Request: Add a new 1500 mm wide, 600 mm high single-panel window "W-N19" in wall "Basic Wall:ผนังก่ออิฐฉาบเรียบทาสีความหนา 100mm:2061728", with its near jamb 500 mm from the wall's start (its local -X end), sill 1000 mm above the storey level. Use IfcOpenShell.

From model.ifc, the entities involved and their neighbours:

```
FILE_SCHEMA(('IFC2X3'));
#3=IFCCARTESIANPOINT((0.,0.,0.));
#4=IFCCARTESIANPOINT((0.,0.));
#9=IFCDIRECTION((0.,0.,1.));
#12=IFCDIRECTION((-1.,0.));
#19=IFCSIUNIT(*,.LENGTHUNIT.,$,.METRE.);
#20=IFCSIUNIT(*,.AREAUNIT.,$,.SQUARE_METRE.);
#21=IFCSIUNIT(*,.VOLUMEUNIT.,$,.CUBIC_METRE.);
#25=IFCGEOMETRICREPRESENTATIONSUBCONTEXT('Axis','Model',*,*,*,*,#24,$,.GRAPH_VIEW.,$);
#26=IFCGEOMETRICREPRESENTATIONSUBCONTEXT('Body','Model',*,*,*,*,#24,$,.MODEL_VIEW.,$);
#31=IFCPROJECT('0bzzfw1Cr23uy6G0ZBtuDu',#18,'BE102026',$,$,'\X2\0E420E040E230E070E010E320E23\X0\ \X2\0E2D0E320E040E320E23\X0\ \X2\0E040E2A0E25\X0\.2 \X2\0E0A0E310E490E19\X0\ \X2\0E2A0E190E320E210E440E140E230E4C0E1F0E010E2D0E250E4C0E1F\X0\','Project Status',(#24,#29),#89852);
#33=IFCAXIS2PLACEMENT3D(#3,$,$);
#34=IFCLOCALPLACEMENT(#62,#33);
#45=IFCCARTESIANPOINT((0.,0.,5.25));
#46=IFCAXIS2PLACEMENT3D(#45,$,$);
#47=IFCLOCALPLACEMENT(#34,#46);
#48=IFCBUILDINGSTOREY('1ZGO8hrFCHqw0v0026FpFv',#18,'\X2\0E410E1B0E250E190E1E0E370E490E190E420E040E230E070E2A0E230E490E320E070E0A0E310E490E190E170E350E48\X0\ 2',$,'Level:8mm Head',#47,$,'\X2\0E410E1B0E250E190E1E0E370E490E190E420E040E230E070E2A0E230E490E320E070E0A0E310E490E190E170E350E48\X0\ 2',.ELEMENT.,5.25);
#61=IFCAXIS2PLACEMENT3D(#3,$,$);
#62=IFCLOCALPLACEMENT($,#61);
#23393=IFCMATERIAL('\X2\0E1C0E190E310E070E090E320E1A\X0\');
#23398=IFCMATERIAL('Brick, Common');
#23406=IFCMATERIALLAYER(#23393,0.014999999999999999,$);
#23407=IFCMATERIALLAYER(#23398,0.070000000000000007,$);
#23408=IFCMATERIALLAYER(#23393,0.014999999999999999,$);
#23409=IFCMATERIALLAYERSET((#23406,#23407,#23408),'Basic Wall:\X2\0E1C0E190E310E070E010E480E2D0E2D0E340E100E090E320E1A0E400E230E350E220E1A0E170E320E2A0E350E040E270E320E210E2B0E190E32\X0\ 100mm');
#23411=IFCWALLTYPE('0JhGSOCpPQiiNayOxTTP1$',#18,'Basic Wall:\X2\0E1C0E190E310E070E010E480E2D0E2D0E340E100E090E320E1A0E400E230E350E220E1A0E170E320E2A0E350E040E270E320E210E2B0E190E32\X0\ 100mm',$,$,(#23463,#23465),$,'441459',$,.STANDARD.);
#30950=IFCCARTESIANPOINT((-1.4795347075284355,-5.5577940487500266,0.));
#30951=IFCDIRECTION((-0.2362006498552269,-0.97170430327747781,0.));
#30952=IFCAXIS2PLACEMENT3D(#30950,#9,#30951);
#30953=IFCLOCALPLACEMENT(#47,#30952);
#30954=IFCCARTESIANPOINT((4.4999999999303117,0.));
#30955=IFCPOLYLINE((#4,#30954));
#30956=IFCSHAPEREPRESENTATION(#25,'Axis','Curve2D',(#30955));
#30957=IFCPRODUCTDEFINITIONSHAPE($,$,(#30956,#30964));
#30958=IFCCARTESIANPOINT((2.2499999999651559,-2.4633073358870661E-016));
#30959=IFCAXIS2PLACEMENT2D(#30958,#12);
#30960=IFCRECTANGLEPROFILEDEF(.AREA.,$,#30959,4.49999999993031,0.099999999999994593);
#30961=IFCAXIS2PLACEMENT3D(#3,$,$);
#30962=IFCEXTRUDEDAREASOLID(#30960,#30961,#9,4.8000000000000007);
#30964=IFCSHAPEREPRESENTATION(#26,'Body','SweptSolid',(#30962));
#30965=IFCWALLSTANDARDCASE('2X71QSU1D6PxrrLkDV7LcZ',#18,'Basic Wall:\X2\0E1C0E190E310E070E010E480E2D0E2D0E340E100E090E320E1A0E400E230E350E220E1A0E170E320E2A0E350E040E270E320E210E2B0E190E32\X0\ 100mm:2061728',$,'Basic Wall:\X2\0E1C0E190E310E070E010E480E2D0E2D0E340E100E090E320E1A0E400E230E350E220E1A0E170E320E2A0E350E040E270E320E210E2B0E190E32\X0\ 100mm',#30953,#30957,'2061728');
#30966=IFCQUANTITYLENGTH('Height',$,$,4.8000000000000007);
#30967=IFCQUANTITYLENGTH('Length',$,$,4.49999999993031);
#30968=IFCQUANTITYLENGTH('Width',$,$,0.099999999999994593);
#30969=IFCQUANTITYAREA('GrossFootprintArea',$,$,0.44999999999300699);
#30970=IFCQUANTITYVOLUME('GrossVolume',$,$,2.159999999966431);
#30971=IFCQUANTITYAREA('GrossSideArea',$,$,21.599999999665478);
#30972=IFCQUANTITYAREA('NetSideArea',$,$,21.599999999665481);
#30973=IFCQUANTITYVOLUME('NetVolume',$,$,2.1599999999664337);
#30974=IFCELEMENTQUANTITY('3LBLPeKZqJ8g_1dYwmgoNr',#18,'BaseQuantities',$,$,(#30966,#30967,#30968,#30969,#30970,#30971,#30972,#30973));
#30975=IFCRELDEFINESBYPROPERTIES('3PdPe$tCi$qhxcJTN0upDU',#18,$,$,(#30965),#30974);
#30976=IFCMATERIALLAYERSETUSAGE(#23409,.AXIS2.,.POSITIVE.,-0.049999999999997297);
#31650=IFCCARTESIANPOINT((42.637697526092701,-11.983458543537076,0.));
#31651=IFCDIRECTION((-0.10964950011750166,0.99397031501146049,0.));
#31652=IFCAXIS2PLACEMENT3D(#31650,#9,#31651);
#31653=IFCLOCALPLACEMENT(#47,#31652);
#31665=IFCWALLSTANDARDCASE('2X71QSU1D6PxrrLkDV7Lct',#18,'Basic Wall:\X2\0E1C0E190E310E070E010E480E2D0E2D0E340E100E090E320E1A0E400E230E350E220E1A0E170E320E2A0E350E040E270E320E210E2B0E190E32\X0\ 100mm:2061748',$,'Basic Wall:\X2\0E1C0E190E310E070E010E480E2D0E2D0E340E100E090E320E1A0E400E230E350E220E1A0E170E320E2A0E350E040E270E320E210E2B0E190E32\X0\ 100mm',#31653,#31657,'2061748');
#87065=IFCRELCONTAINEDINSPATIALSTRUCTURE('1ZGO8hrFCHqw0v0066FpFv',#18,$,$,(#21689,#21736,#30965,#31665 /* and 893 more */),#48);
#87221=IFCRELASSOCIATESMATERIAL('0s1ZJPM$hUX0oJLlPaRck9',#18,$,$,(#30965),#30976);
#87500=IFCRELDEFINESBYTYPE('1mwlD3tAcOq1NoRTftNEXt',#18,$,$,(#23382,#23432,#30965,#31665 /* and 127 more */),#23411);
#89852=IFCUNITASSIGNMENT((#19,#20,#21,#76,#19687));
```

```python
import numpy as np
import ifcopenshell
import ifcopenshell.api.feature
import ifcopenshell.api.geometry
import ifcopenshell.api.pset
import ifcopenshell.api.root
import ifcopenshell.api.spatial
import ifcopenshell.api.type
import ifcopenshell.geom
import ifcopenshell.util.element
import ifcopenshell.util.placement
import ifcopenshell.util.representation
import ifcopenshell.util.shape
import ifcopenshell.util.unit

model = ifcopenshell.open("model.ifc")
unit_scale = ifcopenshell.util.unit.calculate_unit_scale(model)
area_scale = ifcopenshell.util.unit.calculate_unit_scale(model, "AREAUNIT")
volume_scale = ifcopenshell.util.unit.calculate_unit_scale(model, "VOLUMEUNIT")
settings = ifcopenshell.geom.settings()


def volume(element):
    """Net volume in cubic metres, openings subtracted."""
    shape = ifcopenshell.geom.create_shape(settings, element)
    return ifcopenshell.util.shape.get_volume(shape.geometry)


wall = model.by_guid("2X71QSU1D6PxrrLkDV7LcZ")
storey = ifcopenshell.util.element.get_container(wall, ifc_class="IfcBuildingStorey")
context = ifcopenshell.util.representation.get_context(model, "Model", "Body", "MODEL_VIEW")
before = volume(wall)

width, height, from_end, sill = 1.5, 0.6, 0.5, 1  # metres

# The wall runs along its own X axis, and the end named is its -X end.
wall_shape = ifcopenshell.geom.create_shape(settings, wall)
x, y, z = ifcopenshell.util.shape.get_vertices(wall_shape.geometry).T
start = x.min() + from_end
face, thickness = float(y.min()), float(y.max() - y.min())
wall_matrix = ifcopenshell.util.placement.get_local_placement(wall.ObjectPlacement)
level = ifcopenshell.util.placement.get_local_placement(storey.ObjectPlacement)[2, 3]


def in_wall(x, y):
    """Placement at x, y metres in the wall's axes, at sill height."""
    matrix = wall_matrix.copy()
    matrix[:, 3] = wall_matrix @ np.array([x / unit_scale, y / unit_scale, 0.0, 1.0])
    matrix[2, 3] = level + sill / unit_scale
    return matrix


# Opening: a box that overshoots both wall faces by 50 mm.
opening = ifcopenshell.api.root.create_entity(model, ifc_class="IfcOpeningElement")
box = ifcopenshell.api.geometry.add_wall_representation(
    model, context=context, length=width, height=height, thickness=thickness + 0.1
)
ifcopenshell.api.geometry.assign_representation(model, product=opening, representation=box)
ifcopenshell.api.geometry.edit_object_placement(model, product=opening, matrix=in_wall(start, face - 0.05), is_si=False)
ifcopenshell.api.feature.add_feature(model, feature=opening, element=wall)

window = ifcopenshell.api.root.create_entity(model, ifc_class="IfcWindow", name="W-N19")
window.OverallWidth, window.OverallHeight = width / unit_scale, height / unit_scale
body = ifcopenshell.api.geometry.add_window_representation(
    model,
    context=context,
    overall_width=window.OverallWidth,
    overall_height=window.OverallHeight,
    partition_type="SINGLE_PANEL",
)
ifcopenshell.api.geometry.assign_representation(model, product=window, representation=body)
ifcopenshell.api.spatial.assign_container(model, products=[window], relating_structure=storey)
fills = ifcopenshell.api.feature.add_filling(model, opening=opening, element=window)
fills.OwnerHistory = window.OwnerHistory  # required in IFC2X3

# IFC2X3 keeps the operation on the window style.
style = ifcopenshell.api.root.create_entity(model, ifc_class="IfcWindowStyle", name="W-N19")
style.OperationType, style.ConstructionType = "SINGLE_PANEL", "NOTDEFINED"
style.ParameterTakesPrecedence = style.Sizeable = False
ifcopenshell.api.type.assign_type(model, related_objects=[window], relating_type=style)

# Centre the window in the wall's thickness.
ifcopenshell.api.geometry.edit_object_placement(model, product=window, matrix=in_wall(start, face), is_si=False)
window_shape = ifcopenshell.geom.create_shape(settings, window)
depth = ifcopenshell.util.shape.get_vertices(window_shape.geometry)[:, 1]
offset = face + thickness / 2 - (depth.min() + depth.max()) / 2
ifcopenshell.api.geometry.edit_object_placement(model, product=window, matrix=in_wall(start, offset), is_si=False)

after = volume(wall)

# Update the wall's stored quantities.
qto = model.by_id(ifcopenshell.util.element.get_pset(wall, "BaseQuantities", should_inherit=False)["id"])
ifcopenshell.api.pset.edit_qto(model, qto=qto, properties={
    "NetSideArea": after / thickness / area_scale,
    "NetVolume": after / volume_scale,
})

print(f"wall volume {before:.3f} -> {after:.3f} m3")

model.write("model_updated.ifc")
```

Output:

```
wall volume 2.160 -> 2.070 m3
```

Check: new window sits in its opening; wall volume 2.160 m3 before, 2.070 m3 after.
